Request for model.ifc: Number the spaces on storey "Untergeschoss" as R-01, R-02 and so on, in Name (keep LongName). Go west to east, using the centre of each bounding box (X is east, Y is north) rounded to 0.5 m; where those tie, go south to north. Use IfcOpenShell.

First a look at what the model holds.

```python
import ifcopenshell
import ifcopenshell.util.element
import ifcopenshell.util.placement

model = ifcopenshell.open("model.ifc")
print(model.schema)
storey = next(s for s in model.by_type("IfcBuildingStorey") if s.Name == "Untergeschoss")
spaces = [e for e in ifcopenshell.util.element.get_decomposition(storey) if e.is_a("IfcSpace")]
for e in sorted(spaces, key=lambda e: e.id()):
    origin = ifcopenshell.util.placement.get_local_placement(e.ObjectPlacement)[:3, 3]
    print(e.id(), e.Name, e.LongName, origin.round(2) + 0.0, sep=" | ")
```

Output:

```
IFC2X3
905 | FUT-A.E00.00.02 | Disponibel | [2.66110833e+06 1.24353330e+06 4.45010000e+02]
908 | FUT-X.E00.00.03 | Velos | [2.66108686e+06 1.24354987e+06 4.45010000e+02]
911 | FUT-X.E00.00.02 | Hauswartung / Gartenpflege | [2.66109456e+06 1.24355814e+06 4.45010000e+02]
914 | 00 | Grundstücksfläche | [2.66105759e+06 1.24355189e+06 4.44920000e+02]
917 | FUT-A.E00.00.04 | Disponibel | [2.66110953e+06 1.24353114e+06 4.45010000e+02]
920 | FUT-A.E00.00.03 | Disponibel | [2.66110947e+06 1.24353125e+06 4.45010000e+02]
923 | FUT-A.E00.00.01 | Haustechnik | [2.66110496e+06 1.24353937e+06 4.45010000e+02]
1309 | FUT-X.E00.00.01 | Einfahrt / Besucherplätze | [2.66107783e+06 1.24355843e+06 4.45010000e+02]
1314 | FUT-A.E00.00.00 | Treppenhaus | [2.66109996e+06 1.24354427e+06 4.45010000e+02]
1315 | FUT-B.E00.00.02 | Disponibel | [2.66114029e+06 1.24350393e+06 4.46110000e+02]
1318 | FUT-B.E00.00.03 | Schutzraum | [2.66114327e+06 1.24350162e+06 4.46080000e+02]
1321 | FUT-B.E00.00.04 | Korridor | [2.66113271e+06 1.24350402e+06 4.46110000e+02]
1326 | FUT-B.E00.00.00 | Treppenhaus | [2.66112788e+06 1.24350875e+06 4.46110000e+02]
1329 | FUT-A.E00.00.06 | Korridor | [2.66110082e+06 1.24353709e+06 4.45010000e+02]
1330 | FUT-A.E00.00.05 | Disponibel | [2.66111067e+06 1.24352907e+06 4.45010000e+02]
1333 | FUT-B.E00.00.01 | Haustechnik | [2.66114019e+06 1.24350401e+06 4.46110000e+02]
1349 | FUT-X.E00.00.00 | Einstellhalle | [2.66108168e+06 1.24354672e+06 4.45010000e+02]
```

```python
import ifcopenshell
import ifcopenshell.geom
import ifcopenshell.util.element
import ifcopenshell.util.shape

model = ifcopenshell.open("model.ifc")
settings = ifcopenshell.geom.settings()
settings.set("use-world-coords", True)


def centre(element):
    shape = ifcopenshell.geom.create_shape(settings, element)
    return ifcopenshell.util.shape.get_bbox_centroid(shape.geometry)


storey = next(s for s in model.by_type("IfcBuildingStorey") if s.Name == "Untergeschoss")
spaces = [e for e in ifcopenshell.util.element.get_decomposition(storey) if e.is_a("IfcSpace")]

# Insertion points can sit at a corner or the storey origin, so sort by the geometry (in metres).
centres = {e: centre(e) for e in spaces}
spaces.sort(key=lambda e: (round(centres[e][0] / 0.5), centres[e][1]))

for i, e in enumerate(spaces, start=1):
    number = f"R-{i:02d}"
    e.Name = number
    print(e.id(), number)

model.write("model_v2.ifc")
```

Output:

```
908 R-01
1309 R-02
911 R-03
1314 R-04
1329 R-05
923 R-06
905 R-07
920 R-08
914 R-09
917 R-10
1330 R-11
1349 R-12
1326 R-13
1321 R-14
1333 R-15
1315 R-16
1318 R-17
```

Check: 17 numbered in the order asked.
